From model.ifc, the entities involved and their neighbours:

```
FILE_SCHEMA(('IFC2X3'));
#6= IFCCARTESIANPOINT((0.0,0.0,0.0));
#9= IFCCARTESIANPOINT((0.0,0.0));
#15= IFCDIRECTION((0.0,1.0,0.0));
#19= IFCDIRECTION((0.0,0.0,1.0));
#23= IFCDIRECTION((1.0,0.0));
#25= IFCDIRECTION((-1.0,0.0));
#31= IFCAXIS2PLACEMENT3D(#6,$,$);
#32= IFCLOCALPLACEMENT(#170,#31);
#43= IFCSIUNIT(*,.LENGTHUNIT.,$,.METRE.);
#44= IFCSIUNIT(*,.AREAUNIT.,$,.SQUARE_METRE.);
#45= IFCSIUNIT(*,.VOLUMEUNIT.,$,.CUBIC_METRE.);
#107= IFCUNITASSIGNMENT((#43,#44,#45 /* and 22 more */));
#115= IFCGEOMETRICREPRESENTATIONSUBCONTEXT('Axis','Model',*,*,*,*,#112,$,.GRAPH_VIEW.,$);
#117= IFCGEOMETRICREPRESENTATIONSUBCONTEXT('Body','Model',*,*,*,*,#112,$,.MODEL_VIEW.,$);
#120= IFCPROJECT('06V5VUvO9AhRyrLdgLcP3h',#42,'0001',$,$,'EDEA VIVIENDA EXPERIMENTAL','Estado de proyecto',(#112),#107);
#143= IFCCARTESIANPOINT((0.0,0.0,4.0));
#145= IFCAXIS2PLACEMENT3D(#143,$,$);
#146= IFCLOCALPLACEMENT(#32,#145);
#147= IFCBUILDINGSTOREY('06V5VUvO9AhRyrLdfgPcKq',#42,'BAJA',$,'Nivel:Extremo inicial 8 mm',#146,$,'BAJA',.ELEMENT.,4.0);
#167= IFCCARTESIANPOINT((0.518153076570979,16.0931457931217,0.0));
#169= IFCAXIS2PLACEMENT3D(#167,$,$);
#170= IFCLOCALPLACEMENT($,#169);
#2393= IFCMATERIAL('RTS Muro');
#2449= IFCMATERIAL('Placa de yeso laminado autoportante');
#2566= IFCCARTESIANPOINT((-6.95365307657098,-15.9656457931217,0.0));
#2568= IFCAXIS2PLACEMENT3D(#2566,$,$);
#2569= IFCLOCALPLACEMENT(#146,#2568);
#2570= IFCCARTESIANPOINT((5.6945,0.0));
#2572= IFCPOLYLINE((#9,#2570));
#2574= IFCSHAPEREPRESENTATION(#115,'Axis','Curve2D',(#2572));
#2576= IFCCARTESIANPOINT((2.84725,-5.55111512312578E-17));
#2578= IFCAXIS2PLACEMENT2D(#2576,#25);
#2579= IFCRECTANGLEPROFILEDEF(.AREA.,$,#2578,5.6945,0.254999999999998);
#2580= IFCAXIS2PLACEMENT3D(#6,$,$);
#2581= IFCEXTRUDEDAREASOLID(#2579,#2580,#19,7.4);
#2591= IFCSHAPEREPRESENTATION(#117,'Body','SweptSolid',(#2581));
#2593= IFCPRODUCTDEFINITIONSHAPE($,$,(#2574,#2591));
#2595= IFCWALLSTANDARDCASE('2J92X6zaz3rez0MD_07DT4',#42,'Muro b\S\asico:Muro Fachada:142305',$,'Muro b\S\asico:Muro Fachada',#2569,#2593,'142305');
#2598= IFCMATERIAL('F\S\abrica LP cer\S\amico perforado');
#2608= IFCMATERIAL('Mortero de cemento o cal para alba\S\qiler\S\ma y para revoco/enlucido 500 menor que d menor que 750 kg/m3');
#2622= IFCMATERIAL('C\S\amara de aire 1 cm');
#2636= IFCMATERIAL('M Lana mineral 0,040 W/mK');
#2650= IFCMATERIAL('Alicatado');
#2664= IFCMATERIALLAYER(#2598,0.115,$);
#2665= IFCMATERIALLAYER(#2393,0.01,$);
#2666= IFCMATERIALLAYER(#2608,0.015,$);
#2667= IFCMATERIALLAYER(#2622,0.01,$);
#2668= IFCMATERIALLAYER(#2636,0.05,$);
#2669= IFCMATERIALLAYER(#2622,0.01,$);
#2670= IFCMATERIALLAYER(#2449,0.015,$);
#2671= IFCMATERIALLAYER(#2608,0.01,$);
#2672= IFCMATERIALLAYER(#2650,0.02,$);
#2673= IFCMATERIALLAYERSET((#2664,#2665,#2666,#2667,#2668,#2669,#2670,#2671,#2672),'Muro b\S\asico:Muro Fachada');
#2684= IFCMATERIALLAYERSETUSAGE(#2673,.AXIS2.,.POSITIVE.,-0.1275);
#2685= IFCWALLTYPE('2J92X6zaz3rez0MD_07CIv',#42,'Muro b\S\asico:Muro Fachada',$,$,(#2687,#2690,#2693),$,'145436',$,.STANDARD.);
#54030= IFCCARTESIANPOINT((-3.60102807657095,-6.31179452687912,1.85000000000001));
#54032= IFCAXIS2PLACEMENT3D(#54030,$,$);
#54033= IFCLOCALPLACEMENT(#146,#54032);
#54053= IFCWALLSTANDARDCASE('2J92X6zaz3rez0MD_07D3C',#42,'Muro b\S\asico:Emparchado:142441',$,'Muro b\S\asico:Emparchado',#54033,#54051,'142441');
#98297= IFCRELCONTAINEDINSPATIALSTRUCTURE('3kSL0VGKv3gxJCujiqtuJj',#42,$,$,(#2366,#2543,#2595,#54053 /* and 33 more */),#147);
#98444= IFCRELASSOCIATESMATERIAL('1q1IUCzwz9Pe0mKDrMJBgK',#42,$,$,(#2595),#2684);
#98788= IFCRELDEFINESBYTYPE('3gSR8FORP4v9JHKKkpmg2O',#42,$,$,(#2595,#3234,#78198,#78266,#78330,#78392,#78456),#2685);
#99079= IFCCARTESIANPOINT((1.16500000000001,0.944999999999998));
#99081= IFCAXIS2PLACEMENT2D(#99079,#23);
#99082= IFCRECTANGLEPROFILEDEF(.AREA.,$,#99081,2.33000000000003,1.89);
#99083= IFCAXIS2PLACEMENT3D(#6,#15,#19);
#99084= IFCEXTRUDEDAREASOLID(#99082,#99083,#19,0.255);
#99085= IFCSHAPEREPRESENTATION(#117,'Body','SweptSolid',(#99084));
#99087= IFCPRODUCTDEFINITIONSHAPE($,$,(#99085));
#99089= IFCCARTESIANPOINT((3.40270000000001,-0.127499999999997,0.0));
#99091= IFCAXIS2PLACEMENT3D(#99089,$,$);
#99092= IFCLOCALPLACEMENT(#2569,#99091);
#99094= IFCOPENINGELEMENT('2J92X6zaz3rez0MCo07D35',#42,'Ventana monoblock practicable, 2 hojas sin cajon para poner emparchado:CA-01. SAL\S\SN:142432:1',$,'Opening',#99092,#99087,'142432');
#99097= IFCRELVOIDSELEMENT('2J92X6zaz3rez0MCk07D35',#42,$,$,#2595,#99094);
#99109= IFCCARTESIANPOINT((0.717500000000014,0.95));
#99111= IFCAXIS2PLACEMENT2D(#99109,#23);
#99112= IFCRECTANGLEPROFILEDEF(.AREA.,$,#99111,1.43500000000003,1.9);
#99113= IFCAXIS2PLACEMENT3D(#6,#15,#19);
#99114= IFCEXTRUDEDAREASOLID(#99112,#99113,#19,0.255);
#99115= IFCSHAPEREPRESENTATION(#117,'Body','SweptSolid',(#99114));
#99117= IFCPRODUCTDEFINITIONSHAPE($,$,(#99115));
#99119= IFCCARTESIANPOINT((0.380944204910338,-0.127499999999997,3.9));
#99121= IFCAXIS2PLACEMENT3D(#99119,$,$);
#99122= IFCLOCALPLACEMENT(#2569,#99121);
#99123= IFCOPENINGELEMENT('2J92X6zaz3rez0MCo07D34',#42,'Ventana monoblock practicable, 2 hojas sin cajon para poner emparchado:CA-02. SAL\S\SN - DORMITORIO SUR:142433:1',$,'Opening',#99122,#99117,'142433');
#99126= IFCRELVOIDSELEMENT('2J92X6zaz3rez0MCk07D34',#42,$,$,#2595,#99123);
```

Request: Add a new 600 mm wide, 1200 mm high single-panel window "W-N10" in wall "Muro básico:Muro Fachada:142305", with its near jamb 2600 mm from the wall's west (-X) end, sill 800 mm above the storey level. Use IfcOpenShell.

```python
import numpy as np
import ifcopenshell
import ifcopenshell.api.feature
import ifcopenshell.api.geometry
import ifcopenshell.api.root
import ifcopenshell.api.spatial
import ifcopenshell.api.type
import ifcopenshell.geom
import ifcopenshell.util.element
import ifcopenshell.util.placement
import ifcopenshell.util.representation
import ifcopenshell.util.shape
import ifcopenshell.util.unit

model = ifcopenshell.open("model.ifc")
unit_scale = ifcopenshell.util.unit.calculate_unit_scale(model)
settings = ifcopenshell.geom.settings()


def volume(element):
    """Net volume in cubic metres, openings subtracted."""
    shape = ifcopenshell.geom.create_shape(settings, element)
    return ifcopenshell.util.shape.get_volume(shape.geometry)


wall = model.by_guid("2J92X6zaz3rez0MD_07DT4")
storey = ifcopenshell.util.element.get_container(wall, ifc_class="IfcBuildingStorey")
context = ifcopenshell.util.representation.get_context(model, "Model", "Body", "MODEL_VIEW")
before = volume(wall)

width, height, from_end, sill = 0.6, 1.2, 2.6, 0.8  # metres

# The wall runs along its own X axis, and the end named is its -X end.
wall_shape = ifcopenshell.geom.create_shape(settings, wall)
x, y, z = ifcopenshell.util.shape.get_vertices(wall_shape.geometry).T
start = x.min() + from_end
face, thickness = float(y.min()), float(y.max() - y.min())
wall_matrix = ifcopenshell.util.placement.get_local_placement(wall.ObjectPlacement)
level = ifcopenshell.util.placement.get_local_placement(storey.ObjectPlacement)[2, 3]


def in_wall(x, y):
    """Placement at x, y metres in the wall's axes, at sill height."""
    matrix = wall_matrix.copy()
    matrix[:, 3] = wall_matrix @ np.array([x / unit_scale, y / unit_scale, 0.0, 1.0])
    matrix[2, 3] = level + sill / unit_scale
    return matrix


# Opening: a box that overshoots both wall faces by 50 mm.
opening = ifcopenshell.api.root.create_entity(model, ifc_class="IfcOpeningElement")
box = ifcopenshell.api.geometry.add_wall_representation(
    model, context=context, length=width, height=height, thickness=thickness + 0.1
)
ifcopenshell.api.geometry.assign_representation(model, product=opening, representation=box)
ifcopenshell.api.geometry.edit_object_placement(model, product=opening, matrix=in_wall(start, face - 0.05), is_si=False)
ifcopenshell.api.feature.add_feature(model, feature=opening, element=wall)

window = ifcopenshell.api.root.create_entity(model, ifc_class="IfcWindow", name="W-N10")
window.OverallWidth, window.OverallHeight = width / unit_scale, height / unit_scale
body = ifcopenshell.api.geometry.add_window_representation(
    model,
    context=context,
    overall_width=window.OverallWidth,
    overall_height=window.OverallHeight,
    partition_type="SINGLE_PANEL",
)
ifcopenshell.api.geometry.assign_representation(model, product=window, representation=body)
ifcopenshell.api.spatial.assign_container(model, products=[window], relating_structure=storey)
fills = ifcopenshell.api.feature.add_filling(model, opening=opening, element=window)
fills.OwnerHistory = window.OwnerHistory  # required in IFC2X3

# IFC2X3 keeps the operation on the window style.
style = ifcopenshell.api.root.create_entity(model, ifc_class="IfcWindowStyle", name="W-N10")
style.OperationType, style.ConstructionType = "SINGLE_PANEL", "NOTDEFINED"
style.ParameterTakesPrecedence = style.Sizeable = False
ifcopenshell.api.type.assign_type(model, related_objects=[window], relating_type=style)

# Centre the window in the wall's thickness.
ifcopenshell.api.geometry.edit_object_placement(model, product=window, matrix=in_wall(start, face), is_si=False)
window_shape = ifcopenshell.geom.create_shape(settings, window)
depth = ifcopenshell.util.shape.get_vertices(window_shape.geometry)[:, 1]
offset = face + thickness / 2 - (depth.min() + depth.max()) / 2
ifcopenshell.api.geometry.edit_object_placement(model, product=window, matrix=in_wall(start, offset), is_si=False)

after = volume(wall)

print(f"wall volume {before:.3f} -> {after:.3f} m3")

model.write("model_rev.ifc")
```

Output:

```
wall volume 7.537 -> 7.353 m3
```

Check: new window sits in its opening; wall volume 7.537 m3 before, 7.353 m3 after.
